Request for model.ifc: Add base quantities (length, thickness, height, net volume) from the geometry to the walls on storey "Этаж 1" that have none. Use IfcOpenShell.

First a look at what the model holds.

```python
import ifcopenshell
import ifcopenshell.util.element
import ifcopenshell.util.unit

model = ifcopenshell.open("model.ifc")
print(model.schema)
for unit_type in ("LENGTHUNIT", "AREAUNIT", "VOLUMEUNIT"):
    print(unit_type, ifcopenshell.util.unit.calculate_unit_scale(model, unit_type))
storey = next(s for s in model.by_type("IfcBuildingStorey") if s.Name == "Этаж 1")
walls = [e for e in ifcopenshell.util.element.get_decomposition(storey) if e.is_a("IfcWall")]
for e in sorted(walls, key=lambda e: e.id()):
    print(e.id(), e.is_a(), e.Name, list(ifcopenshell.util.element.get_psets(e, qtos_only=True)), sep=" | ")
```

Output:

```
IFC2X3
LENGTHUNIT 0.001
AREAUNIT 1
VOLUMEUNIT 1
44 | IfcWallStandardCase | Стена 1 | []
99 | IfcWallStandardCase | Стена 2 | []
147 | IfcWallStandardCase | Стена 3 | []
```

```python
import ifcopenshell
import ifcopenshell.api.pset
import ifcopenshell.geom
import ifcopenshell.util.element
import ifcopenshell.util.shape
import ifcopenshell.util.unit

model = ifcopenshell.open("model.ifc")
unit_scale = ifcopenshell.util.unit.calculate_unit_scale(model)
volume_scale = ifcopenshell.util.unit.calculate_unit_scale(model, "VOLUMEUNIT")
settings = ifcopenshell.geom.settings()

storey = next(s for s in model.by_type("IfcBuildingStorey") if s.Name == "Этаж 1")
walls = [e for e in ifcopenshell.util.element.get_decomposition(storey) if e.is_a("IfcWall")]

for e in sorted(walls, key=lambda e: e.id()):
    if ifcopenshell.util.element.get_psets(e, qtos_only=True, should_inherit=False):
        continue
    # Geometry comes back in metres, in the element's own axes.
    shape = ifcopenshell.geom.create_shape(settings, e)
    values = {
        "Length": ifcopenshell.util.shape.get_x(shape.geometry) / unit_scale,
        "Width": ifcopenshell.util.shape.get_y(shape.geometry) / unit_scale,
        "Height": ifcopenshell.util.shape.get_z(shape.geometry) / unit_scale,
        "NetVolume": ifcopenshell.util.shape.get_volume(shape.geometry) / volume_scale,
    }
    qto = ifcopenshell.api.pset.add_qto(model, product=e, name="BaseQuantities")
    ifcopenshell.api.pset.edit_qto(model, qto=qto, properties=values)
    print(e.id(), {k: round(v, 3) for k, v in values.items()})

model.write("model-out.ifc")
```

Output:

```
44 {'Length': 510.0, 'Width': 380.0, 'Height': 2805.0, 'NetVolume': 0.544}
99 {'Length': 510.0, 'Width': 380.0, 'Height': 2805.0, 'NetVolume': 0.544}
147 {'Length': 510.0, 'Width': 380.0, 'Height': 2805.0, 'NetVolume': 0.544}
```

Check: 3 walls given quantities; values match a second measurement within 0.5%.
